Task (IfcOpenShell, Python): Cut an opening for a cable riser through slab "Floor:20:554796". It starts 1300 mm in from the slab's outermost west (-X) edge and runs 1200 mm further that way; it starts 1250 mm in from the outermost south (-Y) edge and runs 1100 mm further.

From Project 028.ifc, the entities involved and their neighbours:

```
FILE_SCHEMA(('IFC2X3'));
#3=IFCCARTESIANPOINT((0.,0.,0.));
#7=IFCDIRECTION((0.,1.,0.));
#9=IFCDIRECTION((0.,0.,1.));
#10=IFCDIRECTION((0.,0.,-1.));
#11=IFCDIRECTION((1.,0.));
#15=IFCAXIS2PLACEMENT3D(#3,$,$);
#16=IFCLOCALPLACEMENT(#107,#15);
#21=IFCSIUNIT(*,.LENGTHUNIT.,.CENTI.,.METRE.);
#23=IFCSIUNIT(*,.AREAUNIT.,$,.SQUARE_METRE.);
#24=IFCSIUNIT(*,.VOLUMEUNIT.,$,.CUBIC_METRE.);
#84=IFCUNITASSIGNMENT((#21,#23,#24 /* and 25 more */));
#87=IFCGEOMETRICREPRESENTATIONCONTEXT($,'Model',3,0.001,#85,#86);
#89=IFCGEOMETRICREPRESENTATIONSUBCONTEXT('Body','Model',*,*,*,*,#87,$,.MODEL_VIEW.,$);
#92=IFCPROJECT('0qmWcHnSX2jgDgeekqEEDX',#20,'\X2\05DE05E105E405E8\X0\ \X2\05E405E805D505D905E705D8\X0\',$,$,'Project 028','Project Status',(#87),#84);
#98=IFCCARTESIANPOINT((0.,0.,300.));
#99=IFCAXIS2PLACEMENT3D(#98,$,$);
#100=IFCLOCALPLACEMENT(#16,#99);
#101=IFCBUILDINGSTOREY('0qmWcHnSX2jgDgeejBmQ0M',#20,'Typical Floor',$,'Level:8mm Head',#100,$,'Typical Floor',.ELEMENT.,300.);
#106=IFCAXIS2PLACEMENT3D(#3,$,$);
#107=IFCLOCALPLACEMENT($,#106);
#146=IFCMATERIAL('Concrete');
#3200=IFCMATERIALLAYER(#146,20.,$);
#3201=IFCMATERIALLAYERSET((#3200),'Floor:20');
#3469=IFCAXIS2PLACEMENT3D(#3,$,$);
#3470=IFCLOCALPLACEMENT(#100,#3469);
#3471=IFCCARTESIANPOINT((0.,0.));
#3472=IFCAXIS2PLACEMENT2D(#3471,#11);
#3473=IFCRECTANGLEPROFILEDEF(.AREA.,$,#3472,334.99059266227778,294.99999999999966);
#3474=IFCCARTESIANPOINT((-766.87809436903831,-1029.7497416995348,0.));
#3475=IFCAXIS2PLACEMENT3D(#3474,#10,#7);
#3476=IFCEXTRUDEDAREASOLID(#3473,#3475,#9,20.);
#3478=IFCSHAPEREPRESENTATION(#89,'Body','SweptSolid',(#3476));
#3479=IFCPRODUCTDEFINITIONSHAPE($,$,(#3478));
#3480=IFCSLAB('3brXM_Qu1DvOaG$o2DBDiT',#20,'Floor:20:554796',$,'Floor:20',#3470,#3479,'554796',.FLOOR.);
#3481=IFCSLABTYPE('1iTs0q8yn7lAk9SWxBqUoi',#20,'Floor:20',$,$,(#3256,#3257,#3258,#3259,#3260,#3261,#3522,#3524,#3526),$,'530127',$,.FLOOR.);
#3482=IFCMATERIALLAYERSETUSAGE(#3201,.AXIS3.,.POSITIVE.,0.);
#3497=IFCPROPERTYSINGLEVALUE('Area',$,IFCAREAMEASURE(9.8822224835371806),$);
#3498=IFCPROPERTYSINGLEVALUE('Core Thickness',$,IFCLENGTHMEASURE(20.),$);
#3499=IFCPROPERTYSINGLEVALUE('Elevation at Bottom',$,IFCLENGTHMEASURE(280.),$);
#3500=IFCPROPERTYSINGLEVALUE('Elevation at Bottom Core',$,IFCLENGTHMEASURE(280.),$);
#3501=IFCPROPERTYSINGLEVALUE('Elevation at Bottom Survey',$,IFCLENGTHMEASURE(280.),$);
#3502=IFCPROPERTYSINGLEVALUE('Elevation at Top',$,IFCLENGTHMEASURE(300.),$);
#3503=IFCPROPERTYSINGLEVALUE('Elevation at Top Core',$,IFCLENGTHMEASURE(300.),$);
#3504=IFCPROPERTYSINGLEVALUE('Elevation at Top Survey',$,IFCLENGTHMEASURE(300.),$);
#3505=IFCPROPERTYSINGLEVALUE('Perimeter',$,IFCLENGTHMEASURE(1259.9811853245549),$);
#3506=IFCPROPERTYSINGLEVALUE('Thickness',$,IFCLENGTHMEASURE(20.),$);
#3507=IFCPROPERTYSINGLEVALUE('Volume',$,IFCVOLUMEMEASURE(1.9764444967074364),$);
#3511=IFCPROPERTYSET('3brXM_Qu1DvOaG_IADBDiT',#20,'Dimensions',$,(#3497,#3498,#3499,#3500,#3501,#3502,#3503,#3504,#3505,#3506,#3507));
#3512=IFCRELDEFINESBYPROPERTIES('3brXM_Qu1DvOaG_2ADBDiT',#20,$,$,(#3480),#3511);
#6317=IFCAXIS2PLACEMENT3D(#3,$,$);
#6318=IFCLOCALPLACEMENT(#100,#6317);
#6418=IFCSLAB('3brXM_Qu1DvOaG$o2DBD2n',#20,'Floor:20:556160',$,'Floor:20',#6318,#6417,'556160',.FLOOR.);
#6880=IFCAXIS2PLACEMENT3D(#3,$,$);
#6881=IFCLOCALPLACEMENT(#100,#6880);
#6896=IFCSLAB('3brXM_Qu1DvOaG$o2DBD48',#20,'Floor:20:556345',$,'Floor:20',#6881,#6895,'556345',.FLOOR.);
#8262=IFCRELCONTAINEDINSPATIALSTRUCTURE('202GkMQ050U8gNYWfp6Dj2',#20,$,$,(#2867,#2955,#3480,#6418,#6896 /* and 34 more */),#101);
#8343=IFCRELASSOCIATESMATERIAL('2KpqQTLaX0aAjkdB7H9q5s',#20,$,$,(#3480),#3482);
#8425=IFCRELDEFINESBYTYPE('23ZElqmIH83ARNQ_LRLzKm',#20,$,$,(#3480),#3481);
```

```python
import numpy as np
import ifcopenshell
import ifcopenshell.api.feature
import ifcopenshell.api.geometry
import ifcopenshell.api.pset
import ifcopenshell.api.root
import ifcopenshell.geom
import ifcopenshell.util.element
import ifcopenshell.util.placement
import ifcopenshell.util.representation
import ifcopenshell.util.shape
import ifcopenshell.util.unit

model = ifcopenshell.open("Project 028.ifc")
unit_scale = ifcopenshell.util.unit.calculate_unit_scale(model)
area_scale = ifcopenshell.util.unit.calculate_unit_scale(model, "AREAUNIT")
volume_scale = ifcopenshell.util.unit.calculate_unit_scale(model, "VOLUMEUNIT")
settings = ifcopenshell.geom.settings()


def volume(element):
    """Net volume in cubic metres, openings subtracted."""
    shape = ifcopenshell.geom.create_shape(settings, element)
    return ifcopenshell.util.shape.get_volume(shape.geometry)


slab = model.by_id(3480)
before = volume(slab)

# Extent in the slab's own axes, in metres. The edges named are its -X and -Y sides.
slab_shape = ifcopenshell.geom.create_shape(settings, slab)
vertices = ifcopenshell.util.shape.get_vertices(slab_shape.geometry)
x_min, y_min, bottom = vertices.min(axis=0)
top = vertices[:, 2].max()

opening = ifcopenshell.api.root.create_entity(model, ifc_class="IfcOpeningElement", name="Cable riser opening")
context = ifcopenshell.util.representation.get_context(model, "Model", "Body", "MODEL_VIEW")
width, depth = 1.2, 1.1
outline = [(0.0, 0.0), (width, 0.0), (width, depth), (0.0, depth), (0.0, 0.0)]
# Overshoot both faces by 50 mm so the cut is clean.
shape = ifcopenshell.api.geometry.add_slab_representation(
    model, context=context, depth=top - bottom + 0.1, polyline=outline
)
ifcopenshell.api.geometry.assign_representation(model, product=opening, representation=shape)

matrix = ifcopenshell.util.placement.get_local_placement(slab.ObjectPlacement)
matrix[:, 3] = matrix @ np.append(np.array([x_min + 1.3, y_min + 1.25, bottom - 0.05]) / unit_scale, 1.0)
ifcopenshell.api.geometry.edit_object_placement(model, product=opening, matrix=matrix, is_si=False)
ifcopenshell.api.feature.add_feature(model, feature=opening, element=slab)

after = volume(slab)

# Update the slab's stored quantities.
pset = model.by_id(ifcopenshell.util.element.get_pset(slab, "Dimensions", should_inherit=False)["id"])
ifcopenshell.api.pset.edit_pset(model, pset=pset, properties={
    "Area": model.create_entity("IfcAreaMeasure", after / (top - bottom) / area_scale),
    "Volume": model.create_entity("IfcVolumeMeasure", after / volume_scale),
})

print(f"slab volume {before:.3f} -> {after:.3f} m3")

model.write("Project 028_edited.ifc")
```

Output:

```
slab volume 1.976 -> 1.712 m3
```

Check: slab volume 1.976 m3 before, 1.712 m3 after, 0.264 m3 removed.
